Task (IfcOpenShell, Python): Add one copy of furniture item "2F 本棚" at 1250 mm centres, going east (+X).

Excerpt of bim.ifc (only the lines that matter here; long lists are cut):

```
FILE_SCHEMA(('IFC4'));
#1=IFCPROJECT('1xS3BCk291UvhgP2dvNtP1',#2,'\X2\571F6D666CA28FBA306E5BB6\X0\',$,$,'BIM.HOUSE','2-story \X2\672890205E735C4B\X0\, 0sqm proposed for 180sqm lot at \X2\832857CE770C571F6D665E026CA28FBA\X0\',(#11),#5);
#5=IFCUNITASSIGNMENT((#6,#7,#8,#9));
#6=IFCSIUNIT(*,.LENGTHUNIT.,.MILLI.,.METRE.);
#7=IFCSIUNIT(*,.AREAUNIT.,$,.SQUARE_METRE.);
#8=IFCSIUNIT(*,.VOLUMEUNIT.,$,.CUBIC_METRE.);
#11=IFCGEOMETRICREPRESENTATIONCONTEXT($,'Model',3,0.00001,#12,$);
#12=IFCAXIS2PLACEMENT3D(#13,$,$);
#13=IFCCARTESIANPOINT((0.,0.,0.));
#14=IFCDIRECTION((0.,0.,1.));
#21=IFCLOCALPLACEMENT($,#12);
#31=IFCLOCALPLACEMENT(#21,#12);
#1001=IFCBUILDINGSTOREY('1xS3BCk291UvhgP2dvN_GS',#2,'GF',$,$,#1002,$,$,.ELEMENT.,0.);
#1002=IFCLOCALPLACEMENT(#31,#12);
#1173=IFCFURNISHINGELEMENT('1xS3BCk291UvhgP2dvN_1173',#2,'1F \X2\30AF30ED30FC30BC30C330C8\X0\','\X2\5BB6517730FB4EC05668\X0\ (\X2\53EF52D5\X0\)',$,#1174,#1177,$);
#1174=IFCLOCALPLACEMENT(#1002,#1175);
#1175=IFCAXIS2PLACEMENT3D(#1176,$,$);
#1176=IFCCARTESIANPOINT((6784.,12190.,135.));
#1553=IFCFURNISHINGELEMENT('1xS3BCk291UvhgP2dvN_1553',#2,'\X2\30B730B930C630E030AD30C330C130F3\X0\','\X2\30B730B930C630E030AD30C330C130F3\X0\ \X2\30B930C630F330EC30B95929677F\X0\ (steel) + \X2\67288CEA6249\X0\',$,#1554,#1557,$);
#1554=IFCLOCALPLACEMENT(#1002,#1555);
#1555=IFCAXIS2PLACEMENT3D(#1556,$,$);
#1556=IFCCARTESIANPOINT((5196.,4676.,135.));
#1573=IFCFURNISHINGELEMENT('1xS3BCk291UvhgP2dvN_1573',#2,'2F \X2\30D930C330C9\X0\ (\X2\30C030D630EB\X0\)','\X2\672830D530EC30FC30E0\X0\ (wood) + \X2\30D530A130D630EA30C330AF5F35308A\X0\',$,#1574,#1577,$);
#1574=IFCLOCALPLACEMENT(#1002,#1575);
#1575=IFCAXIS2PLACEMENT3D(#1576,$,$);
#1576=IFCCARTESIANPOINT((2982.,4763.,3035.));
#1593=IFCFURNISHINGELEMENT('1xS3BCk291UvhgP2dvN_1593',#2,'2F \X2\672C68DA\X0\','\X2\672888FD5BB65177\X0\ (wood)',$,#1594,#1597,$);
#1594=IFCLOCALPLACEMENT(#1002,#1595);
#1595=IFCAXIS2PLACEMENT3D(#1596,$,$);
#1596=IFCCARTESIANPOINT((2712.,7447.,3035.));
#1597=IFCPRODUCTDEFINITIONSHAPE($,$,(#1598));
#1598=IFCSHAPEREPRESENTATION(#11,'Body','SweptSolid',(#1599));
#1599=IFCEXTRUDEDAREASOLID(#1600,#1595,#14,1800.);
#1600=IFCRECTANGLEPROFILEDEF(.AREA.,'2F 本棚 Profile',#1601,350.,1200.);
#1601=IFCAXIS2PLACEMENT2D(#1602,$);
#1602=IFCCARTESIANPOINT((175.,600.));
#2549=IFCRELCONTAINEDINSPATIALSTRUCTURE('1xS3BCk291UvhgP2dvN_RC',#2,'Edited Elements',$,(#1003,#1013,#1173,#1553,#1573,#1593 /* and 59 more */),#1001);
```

```python
import numpy as np
import ifcopenshell
import ifcopenshell.api.geometry
import ifcopenshell.api.root
import ifcopenshell.util.element
import ifcopenshell.util.placement

model = ifcopenshell.open("bim.ifc")


def reuse_history(source, copy):
    """copy_class also copies each property set's owner history, people and application; keep the originals."""
    for rel in copy.IsDefinedBy:
        if rel.is_a("IfcRelDefinesByProperties") and (history := rel.RelatingPropertyDefinition.OwnerHistory):
            rel.RelatingPropertyDefinition.OwnerHistory = source.OwnerHistory
            ifcopenshell.util.element.remove_deep2(model, history)


source = model.by_id(1593)
base = ifcopenshell.util.placement.get_local_placement(source.ObjectPlacement)
step = np.array([1.0, 0.0, 0.0]) * 1250.0

for i in range(1, 2):
    copy = ifcopenshell.api.root.copy_class(model, product=source)
    copy.Representation = ifcopenshell.util.element.copy_deep(
        model, source.Representation, exclude=["IfcGeometricRepresentationContext", "IfcRepresentationMap"]
    )
    reuse_history(source, copy)
    matrix = base.copy()
    matrix[:3, 3] += i * step
    print("added at", matrix[:3, 3].round(3) + 0.0)
    ifcopenshell.api.geometry.edit_object_placement(model, product=copy, matrix=matrix, is_si=False)

model.write("bim_rev.ifc")
```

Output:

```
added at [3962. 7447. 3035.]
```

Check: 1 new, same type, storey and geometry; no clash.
